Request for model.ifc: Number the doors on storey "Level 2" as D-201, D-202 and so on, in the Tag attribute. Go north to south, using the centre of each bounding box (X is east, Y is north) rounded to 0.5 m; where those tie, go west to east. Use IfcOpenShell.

First a look at what the model holds.

```python
import ifcopenshell
import ifcopenshell.util.element
import ifcopenshell.util.placement

model = ifcopenshell.open("model.ifc")
print(model.schema)
storey = next(s for s in model.by_type("IfcBuildingStorey") if s.Name == "Level 2")
doors = [e for e in ifcopenshell.util.element.get_decomposition(storey) if e.is_a("IfcDoor")]
for e in sorted(doors, key=lambda e: e.id()):
    origin = ifcopenshell.util.placement.get_local_placement(e.ObjectPlacement)[:3, 3]
    print(e.id(), e.Tag, e.Name, origin.round(2) + 0.0, sep=" | ")
```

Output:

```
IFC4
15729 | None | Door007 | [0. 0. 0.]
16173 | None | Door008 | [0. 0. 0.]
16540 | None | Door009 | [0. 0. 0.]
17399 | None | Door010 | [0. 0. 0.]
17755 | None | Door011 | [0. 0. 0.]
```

```python
import ifcopenshell
import ifcopenshell.geom
import ifcopenshell.util.element
import ifcopenshell.util.shape

model = ifcopenshell.open("model.ifc")
settings = ifcopenshell.geom.settings()
settings.set("use-world-coords", True)


def centre(element):
    shape = ifcopenshell.geom.create_shape(settings, element)
    return ifcopenshell.util.shape.get_bbox_centroid(shape.geometry)


storey = next(s for s in model.by_type("IfcBuildingStorey") if s.Name == "Level 2")
doors = [e for e in ifcopenshell.util.element.get_decomposition(storey) if e.is_a("IfcDoor")]

# Insertion points can sit at a corner or the storey origin, so sort by the geometry (in metres).
centres = {e: centre(e) for e in doors}
doors.sort(key=lambda e: (-round(centres[e][1] / 0.5), centres[e][0]))

for i, e in enumerate(doors, start=1):
    number = f"D-2{i:02d}"
    e.Tag = number
    print(e.id(), number)

model.write("model-out.ifc")
```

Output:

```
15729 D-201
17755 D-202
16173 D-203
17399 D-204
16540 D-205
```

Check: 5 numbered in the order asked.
